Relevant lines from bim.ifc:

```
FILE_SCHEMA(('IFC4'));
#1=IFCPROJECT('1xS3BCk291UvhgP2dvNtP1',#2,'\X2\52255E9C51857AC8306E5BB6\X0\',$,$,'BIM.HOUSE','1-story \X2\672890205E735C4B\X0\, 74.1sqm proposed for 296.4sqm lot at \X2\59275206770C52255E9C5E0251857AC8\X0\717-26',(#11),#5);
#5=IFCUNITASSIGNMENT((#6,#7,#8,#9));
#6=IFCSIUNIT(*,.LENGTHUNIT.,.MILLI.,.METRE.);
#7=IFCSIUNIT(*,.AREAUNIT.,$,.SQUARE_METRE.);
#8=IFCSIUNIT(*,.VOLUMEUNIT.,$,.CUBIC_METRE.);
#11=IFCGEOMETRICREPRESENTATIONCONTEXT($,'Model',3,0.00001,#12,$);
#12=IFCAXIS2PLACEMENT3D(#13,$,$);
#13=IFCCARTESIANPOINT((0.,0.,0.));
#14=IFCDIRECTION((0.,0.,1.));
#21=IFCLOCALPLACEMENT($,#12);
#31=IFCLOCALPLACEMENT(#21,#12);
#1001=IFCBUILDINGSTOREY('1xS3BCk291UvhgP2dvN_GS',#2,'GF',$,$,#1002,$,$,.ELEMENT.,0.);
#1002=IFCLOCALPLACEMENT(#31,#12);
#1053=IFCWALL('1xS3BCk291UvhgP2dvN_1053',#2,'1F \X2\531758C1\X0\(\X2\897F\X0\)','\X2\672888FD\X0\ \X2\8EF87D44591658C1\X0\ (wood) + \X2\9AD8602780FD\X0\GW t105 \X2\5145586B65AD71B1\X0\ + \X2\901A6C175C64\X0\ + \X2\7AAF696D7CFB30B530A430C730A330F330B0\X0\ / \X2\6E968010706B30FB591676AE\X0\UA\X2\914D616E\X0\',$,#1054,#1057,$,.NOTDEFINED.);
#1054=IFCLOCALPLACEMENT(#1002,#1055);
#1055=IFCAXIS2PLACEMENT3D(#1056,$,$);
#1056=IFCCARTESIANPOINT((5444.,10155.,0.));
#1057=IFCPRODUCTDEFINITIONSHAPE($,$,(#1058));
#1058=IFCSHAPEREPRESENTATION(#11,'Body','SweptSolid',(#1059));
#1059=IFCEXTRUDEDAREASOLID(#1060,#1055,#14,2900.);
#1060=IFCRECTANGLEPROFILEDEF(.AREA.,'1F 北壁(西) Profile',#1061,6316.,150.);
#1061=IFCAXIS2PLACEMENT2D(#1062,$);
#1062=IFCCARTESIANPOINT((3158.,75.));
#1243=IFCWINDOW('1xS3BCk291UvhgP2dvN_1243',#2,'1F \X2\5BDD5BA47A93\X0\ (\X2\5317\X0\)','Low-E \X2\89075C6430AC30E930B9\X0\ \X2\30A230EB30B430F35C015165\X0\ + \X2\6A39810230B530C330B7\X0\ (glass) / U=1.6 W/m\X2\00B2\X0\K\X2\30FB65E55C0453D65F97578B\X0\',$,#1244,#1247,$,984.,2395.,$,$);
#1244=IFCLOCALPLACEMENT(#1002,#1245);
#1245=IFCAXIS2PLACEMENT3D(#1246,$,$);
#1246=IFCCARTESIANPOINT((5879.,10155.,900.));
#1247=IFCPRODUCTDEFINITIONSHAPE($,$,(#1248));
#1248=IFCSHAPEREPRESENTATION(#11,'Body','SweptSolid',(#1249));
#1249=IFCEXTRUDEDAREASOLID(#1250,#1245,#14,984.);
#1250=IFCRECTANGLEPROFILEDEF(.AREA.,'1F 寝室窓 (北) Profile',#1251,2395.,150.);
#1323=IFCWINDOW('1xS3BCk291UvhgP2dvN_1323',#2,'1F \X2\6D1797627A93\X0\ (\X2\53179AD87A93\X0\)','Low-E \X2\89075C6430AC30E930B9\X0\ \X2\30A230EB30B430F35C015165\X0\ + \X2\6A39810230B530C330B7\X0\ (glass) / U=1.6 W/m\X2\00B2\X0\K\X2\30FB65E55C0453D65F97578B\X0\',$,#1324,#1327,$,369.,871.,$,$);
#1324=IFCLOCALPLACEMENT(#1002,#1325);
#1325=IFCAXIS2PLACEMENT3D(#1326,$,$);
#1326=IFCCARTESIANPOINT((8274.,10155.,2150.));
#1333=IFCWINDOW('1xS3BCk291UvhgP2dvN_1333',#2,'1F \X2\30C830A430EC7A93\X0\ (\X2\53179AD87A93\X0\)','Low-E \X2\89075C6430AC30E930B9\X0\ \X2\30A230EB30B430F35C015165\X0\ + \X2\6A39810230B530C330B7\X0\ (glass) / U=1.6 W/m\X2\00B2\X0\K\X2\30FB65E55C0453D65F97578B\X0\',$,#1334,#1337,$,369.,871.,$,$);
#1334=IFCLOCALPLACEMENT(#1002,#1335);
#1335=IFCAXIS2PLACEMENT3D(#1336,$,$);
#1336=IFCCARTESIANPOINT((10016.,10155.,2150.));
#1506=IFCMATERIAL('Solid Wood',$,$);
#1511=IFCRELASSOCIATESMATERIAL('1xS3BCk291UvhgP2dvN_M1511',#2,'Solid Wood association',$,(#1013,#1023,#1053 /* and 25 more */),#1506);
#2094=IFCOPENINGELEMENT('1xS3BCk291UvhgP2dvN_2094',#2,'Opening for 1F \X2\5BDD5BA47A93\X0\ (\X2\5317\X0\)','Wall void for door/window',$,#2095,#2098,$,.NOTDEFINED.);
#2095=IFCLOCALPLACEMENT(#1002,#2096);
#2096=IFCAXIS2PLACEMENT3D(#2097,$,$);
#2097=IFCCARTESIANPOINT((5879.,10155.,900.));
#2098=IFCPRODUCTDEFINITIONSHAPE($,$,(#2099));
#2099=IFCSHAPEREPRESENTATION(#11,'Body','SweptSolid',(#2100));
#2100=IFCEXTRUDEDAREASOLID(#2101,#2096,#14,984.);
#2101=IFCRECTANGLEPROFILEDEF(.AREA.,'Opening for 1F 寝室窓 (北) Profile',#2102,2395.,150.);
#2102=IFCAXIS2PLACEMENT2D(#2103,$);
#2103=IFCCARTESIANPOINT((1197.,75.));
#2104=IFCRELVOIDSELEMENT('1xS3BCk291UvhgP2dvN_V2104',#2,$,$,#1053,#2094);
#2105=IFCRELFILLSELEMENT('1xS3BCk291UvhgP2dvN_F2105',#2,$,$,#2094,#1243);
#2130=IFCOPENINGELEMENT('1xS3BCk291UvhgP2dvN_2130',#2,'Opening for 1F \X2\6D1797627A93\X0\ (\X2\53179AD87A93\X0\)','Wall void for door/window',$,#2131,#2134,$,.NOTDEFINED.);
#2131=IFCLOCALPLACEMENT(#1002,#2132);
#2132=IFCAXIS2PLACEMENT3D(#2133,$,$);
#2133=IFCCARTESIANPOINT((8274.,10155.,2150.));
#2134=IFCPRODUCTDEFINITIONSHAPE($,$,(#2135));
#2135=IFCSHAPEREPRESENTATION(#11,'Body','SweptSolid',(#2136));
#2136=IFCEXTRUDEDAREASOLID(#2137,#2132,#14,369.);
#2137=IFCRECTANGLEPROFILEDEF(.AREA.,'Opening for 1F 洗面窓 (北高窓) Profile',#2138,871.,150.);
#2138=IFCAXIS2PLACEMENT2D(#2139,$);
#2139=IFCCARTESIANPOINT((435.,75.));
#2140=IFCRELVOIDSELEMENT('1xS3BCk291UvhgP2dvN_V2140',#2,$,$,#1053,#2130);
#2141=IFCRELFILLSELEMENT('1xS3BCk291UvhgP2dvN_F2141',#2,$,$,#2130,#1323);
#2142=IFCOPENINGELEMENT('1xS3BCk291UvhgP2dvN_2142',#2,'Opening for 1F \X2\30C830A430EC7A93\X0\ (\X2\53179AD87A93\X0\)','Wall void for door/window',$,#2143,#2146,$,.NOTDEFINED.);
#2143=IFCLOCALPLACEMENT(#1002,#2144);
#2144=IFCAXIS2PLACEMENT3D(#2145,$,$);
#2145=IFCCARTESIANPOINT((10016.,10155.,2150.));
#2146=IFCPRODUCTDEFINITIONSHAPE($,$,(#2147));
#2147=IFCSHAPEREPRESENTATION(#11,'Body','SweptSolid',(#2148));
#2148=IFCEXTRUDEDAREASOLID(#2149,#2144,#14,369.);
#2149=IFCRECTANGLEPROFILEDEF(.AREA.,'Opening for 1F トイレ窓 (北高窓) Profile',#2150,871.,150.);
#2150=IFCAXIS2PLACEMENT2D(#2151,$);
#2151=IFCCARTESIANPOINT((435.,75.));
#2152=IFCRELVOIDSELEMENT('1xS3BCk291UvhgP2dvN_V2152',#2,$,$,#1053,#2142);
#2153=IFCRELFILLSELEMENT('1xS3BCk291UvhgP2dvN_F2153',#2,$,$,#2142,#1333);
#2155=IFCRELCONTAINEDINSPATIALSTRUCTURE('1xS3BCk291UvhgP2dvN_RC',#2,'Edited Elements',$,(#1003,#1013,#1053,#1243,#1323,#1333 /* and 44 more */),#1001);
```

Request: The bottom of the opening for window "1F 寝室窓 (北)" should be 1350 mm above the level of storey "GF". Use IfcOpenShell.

```python
import numpy as np
import ifcopenshell
import ifcopenshell.api.geometry
import ifcopenshell.geom
import ifcopenshell.util.element
import ifcopenshell.util.placement
import ifcopenshell.util.shape
import ifcopenshell.util.unit

model = ifcopenshell.open("bim.ifc")
unit_scale = ifcopenshell.util.unit.calculate_unit_scale(model)

window = model.by_guid("1xS3BCk291UvhgP2dvN_1243")
opening = window.FillsVoids[0].RelatingOpeningElement
storey = ifcopenshell.util.element.get_container(window, ifc_class="IfcBuildingStorey")
level = ifcopenshell.util.placement.get_local_placement(storey.ObjectPlacement)[2, 3]

# The opening's origin need not be at the sill, so measure its lowest point.
shape = ifcopenshell.geom.create_shape(ifcopenshell.geom.settings(), opening)
bottom = ifcopenshell.util.shape.get_shape_bottom_elevation(shape, shape.geometry) / unit_scale
dz = level + 1.35 / unit_scale - bottom

shift = np.array([0.0, 0.0, dz])
# The window is not placed relative to its opening, so move both.
for product in (opening, window):
    matrix = ifcopenshell.util.placement.get_local_placement(product.ObjectPlacement)
    matrix[:3, 3] += shift
    ifcopenshell.api.geometry.edit_object_placement(model, product=product, matrix=matrix, is_si=False)

print(f"moved by {dz * unit_scale:+.3f} m")

model.write("bim_rev.ifc")
```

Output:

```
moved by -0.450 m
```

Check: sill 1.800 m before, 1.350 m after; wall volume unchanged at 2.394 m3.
